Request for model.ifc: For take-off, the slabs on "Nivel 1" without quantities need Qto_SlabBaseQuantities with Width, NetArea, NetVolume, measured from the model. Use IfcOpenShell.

First a look at what the model holds.

```python
import ifcopenshell
import ifcopenshell.util.element
import ifcopenshell.util.unit

model = ifcopenshell.open("model.ifc")
print(model.schema)
for unit_type in ("LENGTHUNIT", "AREAUNIT", "VOLUMEUNIT"):
    print(unit_type, ifcopenshell.util.unit.calculate_unit_scale(model, unit_type))
storey = next(s for s in model.by_type("IfcBuildingStorey") if s.Name == "Nivel 1")
slabs = [e for e in ifcopenshell.util.element.get_decomposition(storey) if e.is_a("IfcSlab")]
for e in sorted(slabs, key=lambda e: e.id()):
    print(e.id(), e.is_a(), e.Name, list(ifcopenshell.util.element.get_psets(e, qtos_only=True)), sep=" | ")
```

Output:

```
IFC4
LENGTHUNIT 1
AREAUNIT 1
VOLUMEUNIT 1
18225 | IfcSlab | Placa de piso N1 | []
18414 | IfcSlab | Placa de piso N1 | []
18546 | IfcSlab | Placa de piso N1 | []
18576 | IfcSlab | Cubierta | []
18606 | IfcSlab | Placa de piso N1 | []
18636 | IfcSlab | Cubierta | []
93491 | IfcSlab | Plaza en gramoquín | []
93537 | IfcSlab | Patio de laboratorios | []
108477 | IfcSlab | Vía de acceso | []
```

```python
import ifcopenshell
import ifcopenshell.api.pset
import ifcopenshell.geom
import ifcopenshell.util.element
import ifcopenshell.util.shape
import ifcopenshell.util.unit

model = ifcopenshell.open("model.ifc")
unit_scale = ifcopenshell.util.unit.calculate_unit_scale(model)
area_scale = ifcopenshell.util.unit.calculate_unit_scale(model, "AREAUNIT")
volume_scale = ifcopenshell.util.unit.calculate_unit_scale(model, "VOLUMEUNIT")
settings = ifcopenshell.geom.settings()

storey = next(s for s in model.by_type("IfcBuildingStorey") if s.Name == "Nivel 1")
slabs = [e for e in ifcopenshell.util.element.get_decomposition(storey) if e.is_a("IfcSlab")]

for e in sorted(slabs, key=lambda e: e.id()):
    if ifcopenshell.util.element.get_psets(e, qtos_only=True, should_inherit=False):
        continue
    # Geometry comes back in metres, in the element's own axes.
    shape = ifcopenshell.geom.create_shape(settings, e)
    values = {
        "Width": ifcopenshell.util.shape.get_z(shape.geometry) / unit_scale,
        "NetArea": ifcopenshell.util.shape.get_footprint_area(shape.geometry) / area_scale,
        "NetVolume": ifcopenshell.util.shape.get_volume(shape.geometry) / volume_scale,
    }
    qto = ifcopenshell.api.pset.add_qto(model, product=e, name="Qto_SlabBaseQuantities")
    ifcopenshell.api.pset.edit_qto(model, qto=qto, properties=values)
    print(e.id(), {k: round(v, 3) for k, v in values.items()})

model.write("model-out.ifc")
```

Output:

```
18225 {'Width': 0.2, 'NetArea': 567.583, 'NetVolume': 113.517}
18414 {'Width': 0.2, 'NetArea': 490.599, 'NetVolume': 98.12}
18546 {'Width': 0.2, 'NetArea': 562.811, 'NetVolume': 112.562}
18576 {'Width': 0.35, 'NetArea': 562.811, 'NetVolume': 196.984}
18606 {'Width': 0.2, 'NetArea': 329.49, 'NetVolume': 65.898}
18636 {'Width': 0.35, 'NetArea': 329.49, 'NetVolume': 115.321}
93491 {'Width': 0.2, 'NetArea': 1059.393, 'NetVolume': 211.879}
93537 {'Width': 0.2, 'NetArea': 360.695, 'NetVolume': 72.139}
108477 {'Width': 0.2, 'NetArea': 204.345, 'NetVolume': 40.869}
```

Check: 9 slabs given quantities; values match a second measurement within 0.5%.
